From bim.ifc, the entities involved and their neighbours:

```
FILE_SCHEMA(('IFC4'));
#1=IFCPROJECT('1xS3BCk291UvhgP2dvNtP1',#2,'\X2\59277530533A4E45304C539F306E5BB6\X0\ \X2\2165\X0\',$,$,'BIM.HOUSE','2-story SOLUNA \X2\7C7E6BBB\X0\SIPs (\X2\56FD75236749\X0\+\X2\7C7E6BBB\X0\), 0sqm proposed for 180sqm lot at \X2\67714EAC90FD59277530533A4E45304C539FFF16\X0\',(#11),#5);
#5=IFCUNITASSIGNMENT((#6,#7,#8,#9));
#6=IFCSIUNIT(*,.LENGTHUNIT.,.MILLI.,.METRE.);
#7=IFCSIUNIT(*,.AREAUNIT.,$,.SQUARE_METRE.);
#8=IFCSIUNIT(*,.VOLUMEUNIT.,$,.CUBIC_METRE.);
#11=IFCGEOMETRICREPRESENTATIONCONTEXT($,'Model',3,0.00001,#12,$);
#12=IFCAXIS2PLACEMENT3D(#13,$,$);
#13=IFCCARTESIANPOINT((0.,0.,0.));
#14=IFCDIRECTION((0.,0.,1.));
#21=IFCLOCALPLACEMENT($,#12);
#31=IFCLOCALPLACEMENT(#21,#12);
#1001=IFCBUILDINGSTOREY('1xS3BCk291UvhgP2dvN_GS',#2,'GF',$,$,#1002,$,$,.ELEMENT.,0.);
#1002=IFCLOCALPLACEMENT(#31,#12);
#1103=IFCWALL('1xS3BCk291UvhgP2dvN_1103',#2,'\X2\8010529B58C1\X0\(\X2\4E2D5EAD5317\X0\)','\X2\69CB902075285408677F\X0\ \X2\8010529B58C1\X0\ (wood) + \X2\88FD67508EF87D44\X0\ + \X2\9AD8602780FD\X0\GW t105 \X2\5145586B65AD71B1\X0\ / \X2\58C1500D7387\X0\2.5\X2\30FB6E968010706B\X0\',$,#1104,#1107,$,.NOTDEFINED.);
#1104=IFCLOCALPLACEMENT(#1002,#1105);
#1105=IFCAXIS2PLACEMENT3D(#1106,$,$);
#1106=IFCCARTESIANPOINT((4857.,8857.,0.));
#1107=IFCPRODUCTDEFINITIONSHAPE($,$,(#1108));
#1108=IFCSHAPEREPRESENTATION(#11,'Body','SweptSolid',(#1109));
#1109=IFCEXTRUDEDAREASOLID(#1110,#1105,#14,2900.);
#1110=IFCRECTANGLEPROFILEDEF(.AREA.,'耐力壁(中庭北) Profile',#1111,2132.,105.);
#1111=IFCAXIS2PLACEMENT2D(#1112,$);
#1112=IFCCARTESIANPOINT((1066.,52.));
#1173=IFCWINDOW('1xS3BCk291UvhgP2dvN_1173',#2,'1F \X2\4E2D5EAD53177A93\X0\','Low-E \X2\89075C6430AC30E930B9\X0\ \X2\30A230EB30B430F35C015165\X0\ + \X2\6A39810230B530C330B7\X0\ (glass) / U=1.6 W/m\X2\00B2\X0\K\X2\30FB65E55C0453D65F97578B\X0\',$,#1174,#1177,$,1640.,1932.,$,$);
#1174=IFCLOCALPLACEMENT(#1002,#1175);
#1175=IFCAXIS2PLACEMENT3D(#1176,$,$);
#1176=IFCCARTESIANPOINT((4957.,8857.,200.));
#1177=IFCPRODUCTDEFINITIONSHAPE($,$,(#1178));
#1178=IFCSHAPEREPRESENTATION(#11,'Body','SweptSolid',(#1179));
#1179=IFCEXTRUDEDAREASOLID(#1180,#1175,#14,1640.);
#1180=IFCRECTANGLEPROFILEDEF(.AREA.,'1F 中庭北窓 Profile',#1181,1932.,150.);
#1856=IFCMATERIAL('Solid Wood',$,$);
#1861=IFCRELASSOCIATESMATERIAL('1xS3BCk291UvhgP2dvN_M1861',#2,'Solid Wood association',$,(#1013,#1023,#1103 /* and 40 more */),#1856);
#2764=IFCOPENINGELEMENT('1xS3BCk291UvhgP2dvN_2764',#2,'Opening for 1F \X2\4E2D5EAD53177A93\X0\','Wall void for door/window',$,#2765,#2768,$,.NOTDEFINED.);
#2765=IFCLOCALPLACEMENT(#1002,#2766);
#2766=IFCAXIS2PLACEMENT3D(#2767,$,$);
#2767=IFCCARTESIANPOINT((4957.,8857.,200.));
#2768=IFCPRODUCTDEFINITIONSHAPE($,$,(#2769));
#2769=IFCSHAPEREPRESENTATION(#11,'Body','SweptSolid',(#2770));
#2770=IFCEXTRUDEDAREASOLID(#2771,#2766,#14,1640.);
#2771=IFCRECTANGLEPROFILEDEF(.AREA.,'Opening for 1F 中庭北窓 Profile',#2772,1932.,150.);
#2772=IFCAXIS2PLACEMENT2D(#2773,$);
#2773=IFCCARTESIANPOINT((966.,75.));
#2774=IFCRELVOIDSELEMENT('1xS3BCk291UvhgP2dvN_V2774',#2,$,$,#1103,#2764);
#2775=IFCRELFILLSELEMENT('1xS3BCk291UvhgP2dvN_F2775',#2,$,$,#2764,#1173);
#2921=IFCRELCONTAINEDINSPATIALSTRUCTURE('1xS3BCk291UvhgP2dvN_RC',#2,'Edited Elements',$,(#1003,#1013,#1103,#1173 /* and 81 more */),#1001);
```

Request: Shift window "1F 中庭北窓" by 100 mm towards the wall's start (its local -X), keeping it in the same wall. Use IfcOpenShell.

```python
import ifcopenshell
import ifcopenshell.api.geometry
import ifcopenshell.util.placement

model = ifcopenshell.open("bim.ifc")

window = model.by_guid("1xS3BCk291UvhgP2dvN_1173")
opening = window.FillsVoids[0].RelatingOpeningElement
wall = opening.VoidsElements[0].RelatingBuildingElement

wall_matrix = ifcopenshell.util.placement.get_local_placement(wall.ObjectPlacement)
shift = wall_matrix[:3, 0] * -100.0
before = ifcopenshell.util.placement.get_local_placement(window.ObjectPlacement)[:3, 3].copy()

# The window is not placed relative to its opening, so move both.
for product in (opening, window):
    matrix = ifcopenshell.util.placement.get_local_placement(product.ObjectPlacement)
    matrix[:3, 3] += shift
    ifcopenshell.api.geometry.edit_object_placement(model, product=product, matrix=matrix, is_si=False)

after = ifcopenshell.util.placement.get_local_placement(window.ObjectPlacement)[:3, 3]
print("window moved by", (after - before).round(3) + 0.0)

model.write("bim_v2.ifc")
```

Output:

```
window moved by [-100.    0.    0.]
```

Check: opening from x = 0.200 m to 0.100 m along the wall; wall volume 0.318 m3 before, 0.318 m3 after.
